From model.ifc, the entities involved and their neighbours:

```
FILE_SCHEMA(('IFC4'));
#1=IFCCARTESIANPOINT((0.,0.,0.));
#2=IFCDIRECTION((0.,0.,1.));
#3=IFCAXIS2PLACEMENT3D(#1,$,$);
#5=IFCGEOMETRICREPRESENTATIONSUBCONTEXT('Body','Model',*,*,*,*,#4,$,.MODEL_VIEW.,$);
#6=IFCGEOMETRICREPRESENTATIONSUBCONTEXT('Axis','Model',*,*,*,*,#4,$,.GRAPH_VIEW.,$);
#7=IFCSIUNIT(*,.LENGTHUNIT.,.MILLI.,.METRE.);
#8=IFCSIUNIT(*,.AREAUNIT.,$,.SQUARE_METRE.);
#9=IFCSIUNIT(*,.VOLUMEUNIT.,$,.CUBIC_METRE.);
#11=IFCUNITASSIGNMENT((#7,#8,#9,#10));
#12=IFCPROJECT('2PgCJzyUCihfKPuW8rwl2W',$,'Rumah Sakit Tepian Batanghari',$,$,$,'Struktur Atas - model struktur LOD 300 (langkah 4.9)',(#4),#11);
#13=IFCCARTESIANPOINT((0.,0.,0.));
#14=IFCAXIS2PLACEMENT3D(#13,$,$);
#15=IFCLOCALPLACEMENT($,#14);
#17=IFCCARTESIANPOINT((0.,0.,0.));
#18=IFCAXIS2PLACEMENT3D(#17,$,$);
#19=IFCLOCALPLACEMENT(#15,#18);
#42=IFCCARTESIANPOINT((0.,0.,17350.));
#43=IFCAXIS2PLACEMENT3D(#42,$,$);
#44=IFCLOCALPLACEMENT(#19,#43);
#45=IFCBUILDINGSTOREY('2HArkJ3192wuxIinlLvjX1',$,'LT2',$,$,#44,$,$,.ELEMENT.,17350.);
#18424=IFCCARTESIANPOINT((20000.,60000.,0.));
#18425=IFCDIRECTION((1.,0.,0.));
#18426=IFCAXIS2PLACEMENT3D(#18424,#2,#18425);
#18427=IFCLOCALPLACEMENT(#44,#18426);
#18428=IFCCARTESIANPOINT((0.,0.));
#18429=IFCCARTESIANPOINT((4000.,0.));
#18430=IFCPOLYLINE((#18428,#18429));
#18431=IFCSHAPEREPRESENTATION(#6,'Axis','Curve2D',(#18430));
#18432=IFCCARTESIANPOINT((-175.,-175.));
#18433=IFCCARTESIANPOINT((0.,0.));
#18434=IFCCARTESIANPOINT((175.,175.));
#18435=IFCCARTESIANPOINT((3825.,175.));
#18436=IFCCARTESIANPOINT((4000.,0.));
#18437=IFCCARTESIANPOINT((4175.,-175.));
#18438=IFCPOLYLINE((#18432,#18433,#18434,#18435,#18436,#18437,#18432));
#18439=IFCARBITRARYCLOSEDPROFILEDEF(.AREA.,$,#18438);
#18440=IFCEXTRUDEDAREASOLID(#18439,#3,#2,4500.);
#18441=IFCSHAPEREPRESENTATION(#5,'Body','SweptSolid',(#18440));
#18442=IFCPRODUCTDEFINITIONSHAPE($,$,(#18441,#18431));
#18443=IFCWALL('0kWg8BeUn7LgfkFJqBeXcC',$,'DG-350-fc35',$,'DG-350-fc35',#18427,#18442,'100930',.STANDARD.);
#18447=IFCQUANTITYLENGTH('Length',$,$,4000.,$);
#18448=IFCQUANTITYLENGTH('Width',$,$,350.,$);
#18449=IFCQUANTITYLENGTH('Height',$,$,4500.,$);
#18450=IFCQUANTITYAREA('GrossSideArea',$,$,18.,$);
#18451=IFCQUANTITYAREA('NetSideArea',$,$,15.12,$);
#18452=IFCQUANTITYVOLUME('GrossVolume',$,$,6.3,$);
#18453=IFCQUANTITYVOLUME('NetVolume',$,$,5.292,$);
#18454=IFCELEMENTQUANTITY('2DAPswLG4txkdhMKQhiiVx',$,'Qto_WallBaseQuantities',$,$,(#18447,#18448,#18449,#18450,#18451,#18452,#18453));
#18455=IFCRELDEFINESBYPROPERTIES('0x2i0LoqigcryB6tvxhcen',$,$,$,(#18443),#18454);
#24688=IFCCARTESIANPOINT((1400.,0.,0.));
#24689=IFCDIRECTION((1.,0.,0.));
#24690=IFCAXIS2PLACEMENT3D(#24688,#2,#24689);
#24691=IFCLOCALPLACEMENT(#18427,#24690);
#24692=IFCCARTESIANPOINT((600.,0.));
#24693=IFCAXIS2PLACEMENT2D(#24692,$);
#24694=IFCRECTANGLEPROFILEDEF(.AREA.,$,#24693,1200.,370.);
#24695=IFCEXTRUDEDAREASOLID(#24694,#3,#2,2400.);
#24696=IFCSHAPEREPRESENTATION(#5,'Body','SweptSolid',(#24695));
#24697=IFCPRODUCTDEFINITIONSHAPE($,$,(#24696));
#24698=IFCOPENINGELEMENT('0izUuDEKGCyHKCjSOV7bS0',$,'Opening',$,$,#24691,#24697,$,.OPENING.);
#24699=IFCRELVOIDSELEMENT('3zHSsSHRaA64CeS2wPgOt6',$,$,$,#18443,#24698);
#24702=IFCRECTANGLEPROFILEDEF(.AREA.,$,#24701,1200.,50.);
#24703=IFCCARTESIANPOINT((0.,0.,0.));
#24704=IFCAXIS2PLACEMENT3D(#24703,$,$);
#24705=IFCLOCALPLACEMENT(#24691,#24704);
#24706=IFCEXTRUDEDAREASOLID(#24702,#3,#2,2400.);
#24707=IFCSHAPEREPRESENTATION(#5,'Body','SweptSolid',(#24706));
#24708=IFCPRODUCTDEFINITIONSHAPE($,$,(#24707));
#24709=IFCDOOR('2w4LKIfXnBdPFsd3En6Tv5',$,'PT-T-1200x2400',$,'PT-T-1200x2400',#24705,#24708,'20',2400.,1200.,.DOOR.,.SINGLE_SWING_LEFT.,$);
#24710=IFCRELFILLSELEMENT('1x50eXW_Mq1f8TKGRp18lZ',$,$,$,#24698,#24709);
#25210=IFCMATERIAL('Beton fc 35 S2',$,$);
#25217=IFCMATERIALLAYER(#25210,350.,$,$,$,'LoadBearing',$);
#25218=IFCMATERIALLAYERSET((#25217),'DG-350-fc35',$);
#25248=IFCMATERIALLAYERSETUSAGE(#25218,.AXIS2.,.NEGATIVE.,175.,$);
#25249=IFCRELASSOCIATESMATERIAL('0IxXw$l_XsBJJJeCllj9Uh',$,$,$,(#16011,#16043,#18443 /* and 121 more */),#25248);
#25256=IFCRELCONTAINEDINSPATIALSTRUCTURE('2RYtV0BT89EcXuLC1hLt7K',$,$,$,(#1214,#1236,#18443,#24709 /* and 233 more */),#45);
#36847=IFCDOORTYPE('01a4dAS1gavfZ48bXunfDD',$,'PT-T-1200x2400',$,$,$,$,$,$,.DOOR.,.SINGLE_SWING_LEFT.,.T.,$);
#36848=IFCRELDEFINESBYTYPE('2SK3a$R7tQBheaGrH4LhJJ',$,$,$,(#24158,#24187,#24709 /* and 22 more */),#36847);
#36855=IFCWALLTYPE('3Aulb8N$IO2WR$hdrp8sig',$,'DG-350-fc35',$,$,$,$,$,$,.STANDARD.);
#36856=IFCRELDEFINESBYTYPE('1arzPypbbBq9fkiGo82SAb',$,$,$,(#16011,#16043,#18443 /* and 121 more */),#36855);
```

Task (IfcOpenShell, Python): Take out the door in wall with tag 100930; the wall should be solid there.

```python
import ifcopenshell
import ifcopenshell.api.feature
import ifcopenshell.api.pset
import ifcopenshell.api.root
import ifcopenshell.geom
import ifcopenshell.util.element
import ifcopenshell.util.shape
import ifcopenshell.util.unit

model = ifcopenshell.open("model.ifc")
area_scale = ifcopenshell.util.unit.calculate_unit_scale(model, "AREAUNIT")
volume_scale = ifcopenshell.util.unit.calculate_unit_scale(model, "VOLUMEUNIT")
settings = ifcopenshell.geom.settings()


def volume(element):
    """Net volume in cubic metres, openings subtracted."""
    shape = ifcopenshell.geom.create_shape(settings, element)
    return ifcopenshell.util.shape.get_volume(shape.geometry)


door = model.by_guid("2w4LKIfXnBdPFsd3En6Tv5")
opening = door.FillsVoids[0].RelatingOpeningElement
wall = opening.VoidsElements[0].RelatingBuildingElement
before = volume(wall)

ifcopenshell.api.root.remove_product(model, product=door)
ifcopenshell.api.feature.remove_feature(model, feature=opening)

after = volume(wall)
thickness = 0.35  # wall thickness in metres

# Update the wall's stored quantities.
qto = model.by_id(ifcopenshell.util.element.get_pset(wall, "Qto_WallBaseQuantities", should_inherit=False)["id"])
ifcopenshell.api.pset.edit_qto(model, qto=qto, properties={
    "NetSideArea": after / thickness / area_scale,
    "NetVolume": after / volume_scale,
})

print(f"wall volume {before:.3f} -> {after:.3f} m3")

model.write("model_v2.ifc")
```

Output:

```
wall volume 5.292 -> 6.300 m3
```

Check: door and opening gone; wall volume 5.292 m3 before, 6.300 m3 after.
